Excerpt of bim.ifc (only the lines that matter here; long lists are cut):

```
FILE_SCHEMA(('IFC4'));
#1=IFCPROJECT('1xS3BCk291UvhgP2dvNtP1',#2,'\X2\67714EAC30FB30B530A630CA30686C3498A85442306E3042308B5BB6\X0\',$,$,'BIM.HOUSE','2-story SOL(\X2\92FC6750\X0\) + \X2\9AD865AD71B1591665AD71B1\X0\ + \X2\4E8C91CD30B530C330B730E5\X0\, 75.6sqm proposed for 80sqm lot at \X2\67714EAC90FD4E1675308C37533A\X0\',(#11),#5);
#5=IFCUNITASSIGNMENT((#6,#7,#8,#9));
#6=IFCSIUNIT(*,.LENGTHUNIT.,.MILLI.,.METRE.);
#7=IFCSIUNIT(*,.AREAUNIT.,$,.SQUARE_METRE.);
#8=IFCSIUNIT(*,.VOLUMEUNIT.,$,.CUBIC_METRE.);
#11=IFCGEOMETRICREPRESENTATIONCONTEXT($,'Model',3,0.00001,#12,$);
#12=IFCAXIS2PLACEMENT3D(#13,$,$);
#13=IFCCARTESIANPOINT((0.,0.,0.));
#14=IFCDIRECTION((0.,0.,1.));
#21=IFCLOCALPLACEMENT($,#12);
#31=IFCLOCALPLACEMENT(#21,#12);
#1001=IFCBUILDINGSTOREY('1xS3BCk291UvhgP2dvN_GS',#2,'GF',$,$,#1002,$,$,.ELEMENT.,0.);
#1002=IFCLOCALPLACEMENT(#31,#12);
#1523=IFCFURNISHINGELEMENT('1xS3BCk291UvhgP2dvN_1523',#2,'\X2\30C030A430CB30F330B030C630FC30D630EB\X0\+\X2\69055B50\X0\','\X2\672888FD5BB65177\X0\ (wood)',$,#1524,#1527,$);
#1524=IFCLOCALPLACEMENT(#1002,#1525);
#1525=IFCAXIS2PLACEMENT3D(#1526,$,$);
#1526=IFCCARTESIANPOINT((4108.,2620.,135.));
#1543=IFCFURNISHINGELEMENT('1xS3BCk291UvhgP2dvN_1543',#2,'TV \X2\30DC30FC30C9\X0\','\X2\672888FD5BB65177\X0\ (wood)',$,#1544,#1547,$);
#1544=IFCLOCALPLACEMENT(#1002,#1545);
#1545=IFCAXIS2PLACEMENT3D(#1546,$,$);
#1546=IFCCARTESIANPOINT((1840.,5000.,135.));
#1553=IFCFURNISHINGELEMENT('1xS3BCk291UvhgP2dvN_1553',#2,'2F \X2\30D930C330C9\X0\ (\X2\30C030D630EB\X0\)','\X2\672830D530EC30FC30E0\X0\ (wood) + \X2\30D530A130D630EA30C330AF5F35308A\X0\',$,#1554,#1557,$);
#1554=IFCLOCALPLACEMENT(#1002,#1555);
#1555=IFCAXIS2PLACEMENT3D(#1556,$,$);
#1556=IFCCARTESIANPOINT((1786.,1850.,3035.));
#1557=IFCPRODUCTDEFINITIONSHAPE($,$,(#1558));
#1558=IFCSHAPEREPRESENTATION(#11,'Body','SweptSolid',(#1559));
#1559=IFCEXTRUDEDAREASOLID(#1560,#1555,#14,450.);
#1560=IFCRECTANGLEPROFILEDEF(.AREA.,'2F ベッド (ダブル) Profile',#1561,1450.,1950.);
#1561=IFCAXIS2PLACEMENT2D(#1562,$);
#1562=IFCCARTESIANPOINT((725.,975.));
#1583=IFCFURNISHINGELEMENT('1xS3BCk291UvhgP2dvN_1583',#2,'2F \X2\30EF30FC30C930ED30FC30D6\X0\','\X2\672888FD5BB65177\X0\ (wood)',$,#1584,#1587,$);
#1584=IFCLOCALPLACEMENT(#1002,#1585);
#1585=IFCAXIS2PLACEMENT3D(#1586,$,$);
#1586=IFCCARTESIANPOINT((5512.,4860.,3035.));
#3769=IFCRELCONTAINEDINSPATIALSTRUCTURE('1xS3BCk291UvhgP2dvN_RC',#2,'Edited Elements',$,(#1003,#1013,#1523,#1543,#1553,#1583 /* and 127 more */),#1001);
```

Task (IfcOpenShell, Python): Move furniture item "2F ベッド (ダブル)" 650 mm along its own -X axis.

```python
import ifcopenshell
import ifcopenshell.api.geometry
import ifcopenshell.util.placement

model = ifcopenshell.open("bim.ifc")

item = model.by_id(1553)
matrix = ifcopenshell.util.placement.get_local_placement(item.ObjectPlacement)
matrix[:3, 3] -= matrix[:3, 0] * 650.0
ifcopenshell.api.geometry.edit_object_placement(model, product=item, matrix=matrix, is_si=False)

print(ifcopenshell.util.placement.get_local_placement(item.ObjectPlacement).round(3) + 0.0)

model.write("bim_v2.ifc")
```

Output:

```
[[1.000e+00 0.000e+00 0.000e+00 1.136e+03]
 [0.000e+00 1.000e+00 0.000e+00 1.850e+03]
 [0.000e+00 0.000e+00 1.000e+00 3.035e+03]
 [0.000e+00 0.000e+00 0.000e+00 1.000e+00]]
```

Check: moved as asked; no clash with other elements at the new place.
